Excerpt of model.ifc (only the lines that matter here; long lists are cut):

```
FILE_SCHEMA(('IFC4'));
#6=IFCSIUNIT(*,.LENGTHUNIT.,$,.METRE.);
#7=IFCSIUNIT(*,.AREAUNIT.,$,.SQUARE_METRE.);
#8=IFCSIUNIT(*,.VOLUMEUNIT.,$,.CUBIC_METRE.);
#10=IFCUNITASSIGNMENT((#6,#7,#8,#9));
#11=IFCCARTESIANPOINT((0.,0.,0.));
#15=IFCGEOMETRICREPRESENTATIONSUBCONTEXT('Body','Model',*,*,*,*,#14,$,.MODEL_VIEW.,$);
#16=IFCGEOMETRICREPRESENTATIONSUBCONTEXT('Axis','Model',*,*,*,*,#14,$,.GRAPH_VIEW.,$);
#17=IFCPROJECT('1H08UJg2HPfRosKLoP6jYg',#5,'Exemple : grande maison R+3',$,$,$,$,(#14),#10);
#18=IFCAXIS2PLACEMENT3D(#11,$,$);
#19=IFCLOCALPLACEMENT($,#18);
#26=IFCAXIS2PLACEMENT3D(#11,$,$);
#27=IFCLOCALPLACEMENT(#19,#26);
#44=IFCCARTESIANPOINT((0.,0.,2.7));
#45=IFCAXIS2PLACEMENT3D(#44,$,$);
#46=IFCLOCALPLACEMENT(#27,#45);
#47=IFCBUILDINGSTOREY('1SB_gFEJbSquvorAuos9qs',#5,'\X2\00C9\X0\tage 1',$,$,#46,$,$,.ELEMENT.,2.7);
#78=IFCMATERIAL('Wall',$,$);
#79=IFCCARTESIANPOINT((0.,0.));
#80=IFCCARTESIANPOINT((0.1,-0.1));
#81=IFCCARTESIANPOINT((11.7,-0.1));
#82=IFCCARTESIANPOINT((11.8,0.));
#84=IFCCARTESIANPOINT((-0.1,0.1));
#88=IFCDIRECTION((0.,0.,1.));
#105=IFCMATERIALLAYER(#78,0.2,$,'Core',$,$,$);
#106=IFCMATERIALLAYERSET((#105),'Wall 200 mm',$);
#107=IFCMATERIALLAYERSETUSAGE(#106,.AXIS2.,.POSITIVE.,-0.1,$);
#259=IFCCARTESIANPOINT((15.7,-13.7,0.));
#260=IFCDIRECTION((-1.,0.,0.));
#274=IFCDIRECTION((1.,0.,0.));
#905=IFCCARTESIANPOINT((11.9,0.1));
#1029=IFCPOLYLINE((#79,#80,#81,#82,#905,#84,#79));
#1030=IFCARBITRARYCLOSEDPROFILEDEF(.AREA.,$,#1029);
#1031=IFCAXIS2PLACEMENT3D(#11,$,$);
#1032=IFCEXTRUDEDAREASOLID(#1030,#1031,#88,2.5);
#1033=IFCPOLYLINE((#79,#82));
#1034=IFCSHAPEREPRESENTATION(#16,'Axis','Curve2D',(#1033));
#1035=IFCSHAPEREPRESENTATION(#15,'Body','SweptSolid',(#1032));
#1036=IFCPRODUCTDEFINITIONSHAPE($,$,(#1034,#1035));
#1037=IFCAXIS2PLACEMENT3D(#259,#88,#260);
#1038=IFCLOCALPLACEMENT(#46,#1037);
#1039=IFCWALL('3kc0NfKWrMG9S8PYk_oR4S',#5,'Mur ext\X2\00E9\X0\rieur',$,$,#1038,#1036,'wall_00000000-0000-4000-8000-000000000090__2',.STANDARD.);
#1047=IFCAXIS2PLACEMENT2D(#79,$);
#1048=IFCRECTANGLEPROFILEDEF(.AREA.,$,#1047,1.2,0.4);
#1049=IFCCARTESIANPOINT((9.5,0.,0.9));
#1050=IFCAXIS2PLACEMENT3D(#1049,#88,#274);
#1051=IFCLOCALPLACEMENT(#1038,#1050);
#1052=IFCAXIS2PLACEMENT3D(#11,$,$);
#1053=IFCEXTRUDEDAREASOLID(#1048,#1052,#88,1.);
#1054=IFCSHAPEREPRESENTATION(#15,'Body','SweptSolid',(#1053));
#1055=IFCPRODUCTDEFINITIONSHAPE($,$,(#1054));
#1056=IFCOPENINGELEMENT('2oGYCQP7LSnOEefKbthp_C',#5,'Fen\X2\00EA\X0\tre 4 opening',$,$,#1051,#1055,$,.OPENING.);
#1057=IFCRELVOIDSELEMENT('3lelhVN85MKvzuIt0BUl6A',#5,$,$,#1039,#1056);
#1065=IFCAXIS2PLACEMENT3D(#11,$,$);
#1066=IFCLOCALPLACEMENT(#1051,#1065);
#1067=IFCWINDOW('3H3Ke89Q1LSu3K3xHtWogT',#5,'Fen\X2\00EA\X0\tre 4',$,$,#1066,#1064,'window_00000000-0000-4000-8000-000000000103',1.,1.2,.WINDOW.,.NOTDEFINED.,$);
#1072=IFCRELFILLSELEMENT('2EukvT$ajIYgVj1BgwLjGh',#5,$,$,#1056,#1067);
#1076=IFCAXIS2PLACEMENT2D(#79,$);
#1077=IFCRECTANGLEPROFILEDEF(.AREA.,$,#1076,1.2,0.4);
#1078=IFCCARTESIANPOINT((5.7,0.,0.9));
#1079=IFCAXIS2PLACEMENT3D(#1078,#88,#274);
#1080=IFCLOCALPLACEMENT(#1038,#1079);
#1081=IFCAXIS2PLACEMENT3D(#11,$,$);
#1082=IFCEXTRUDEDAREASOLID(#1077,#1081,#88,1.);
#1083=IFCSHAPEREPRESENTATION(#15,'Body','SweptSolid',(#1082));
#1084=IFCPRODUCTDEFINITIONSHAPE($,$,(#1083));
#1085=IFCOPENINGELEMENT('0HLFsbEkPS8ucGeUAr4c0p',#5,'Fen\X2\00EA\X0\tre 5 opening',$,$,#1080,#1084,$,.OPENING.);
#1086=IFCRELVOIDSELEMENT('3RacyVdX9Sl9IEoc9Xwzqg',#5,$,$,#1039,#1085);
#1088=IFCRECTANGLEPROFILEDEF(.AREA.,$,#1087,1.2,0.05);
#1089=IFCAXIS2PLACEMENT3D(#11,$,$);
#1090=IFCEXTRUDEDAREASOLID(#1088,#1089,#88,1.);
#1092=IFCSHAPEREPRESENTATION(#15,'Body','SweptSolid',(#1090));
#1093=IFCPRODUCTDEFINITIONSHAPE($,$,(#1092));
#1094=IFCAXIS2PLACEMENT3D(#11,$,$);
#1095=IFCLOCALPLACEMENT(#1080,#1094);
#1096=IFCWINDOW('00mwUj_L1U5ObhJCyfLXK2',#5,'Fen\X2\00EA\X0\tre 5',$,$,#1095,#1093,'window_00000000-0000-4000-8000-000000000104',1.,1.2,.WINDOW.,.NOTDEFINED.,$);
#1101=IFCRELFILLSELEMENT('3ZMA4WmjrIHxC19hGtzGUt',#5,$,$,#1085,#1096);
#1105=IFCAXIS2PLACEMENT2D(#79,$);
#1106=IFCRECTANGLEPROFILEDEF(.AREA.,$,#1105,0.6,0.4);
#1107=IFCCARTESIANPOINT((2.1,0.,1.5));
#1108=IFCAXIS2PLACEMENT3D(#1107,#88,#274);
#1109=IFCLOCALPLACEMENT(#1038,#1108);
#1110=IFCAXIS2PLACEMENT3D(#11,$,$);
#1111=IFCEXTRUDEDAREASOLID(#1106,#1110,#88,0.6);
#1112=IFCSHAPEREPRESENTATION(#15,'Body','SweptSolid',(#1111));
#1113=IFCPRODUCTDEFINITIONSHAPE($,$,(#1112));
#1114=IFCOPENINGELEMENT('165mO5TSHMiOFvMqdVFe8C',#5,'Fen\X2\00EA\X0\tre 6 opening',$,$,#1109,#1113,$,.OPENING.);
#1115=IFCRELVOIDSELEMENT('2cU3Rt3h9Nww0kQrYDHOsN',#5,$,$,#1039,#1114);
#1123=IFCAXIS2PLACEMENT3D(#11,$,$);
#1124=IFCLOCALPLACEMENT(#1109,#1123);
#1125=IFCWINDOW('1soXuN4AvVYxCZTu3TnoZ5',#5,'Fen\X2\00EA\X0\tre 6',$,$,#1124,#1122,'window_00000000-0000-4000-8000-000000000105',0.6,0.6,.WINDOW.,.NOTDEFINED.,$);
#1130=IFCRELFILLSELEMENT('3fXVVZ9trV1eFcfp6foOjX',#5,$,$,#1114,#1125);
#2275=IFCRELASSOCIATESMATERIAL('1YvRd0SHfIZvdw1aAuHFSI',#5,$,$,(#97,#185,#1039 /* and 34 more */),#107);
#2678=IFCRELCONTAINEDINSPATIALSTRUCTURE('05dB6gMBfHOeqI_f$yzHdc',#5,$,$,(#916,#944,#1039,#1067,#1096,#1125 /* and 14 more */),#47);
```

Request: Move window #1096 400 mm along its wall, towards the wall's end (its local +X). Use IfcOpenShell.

```python
import ifcopenshell
import ifcopenshell.api.geometry
import ifcopenshell.util.placement

model = ifcopenshell.open("model.ifc")

window = model.by_guid("00mwUj_L1U5ObhJCyfLXK2")
opening = window.FillsVoids[0].RelatingOpeningElement
wall = opening.VoidsElements[0].RelatingBuildingElement

wall_matrix = ifcopenshell.util.placement.get_local_placement(wall.ObjectPlacement)
shift = wall_matrix[:3, 0] * 0.4
before = ifcopenshell.util.placement.get_local_placement(window.ObjectPlacement)[:3, 3].copy()

# The window is placed relative to its opening, so it follows when the opening moves.
matrix = ifcopenshell.util.placement.get_local_placement(opening.ObjectPlacement)
matrix[:3, 3] += shift
ifcopenshell.api.geometry.edit_object_placement(
    model, product=opening, matrix=matrix, is_si=False, should_transform_children=True
)

after = ifcopenshell.util.placement.get_local_placement(window.ObjectPlacement)[:3, 3]
print("window moved by", (after - before).round(3) + 0.0)

model.write("model_rev.ifc")
```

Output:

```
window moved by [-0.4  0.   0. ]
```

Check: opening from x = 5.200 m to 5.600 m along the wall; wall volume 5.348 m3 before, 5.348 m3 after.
